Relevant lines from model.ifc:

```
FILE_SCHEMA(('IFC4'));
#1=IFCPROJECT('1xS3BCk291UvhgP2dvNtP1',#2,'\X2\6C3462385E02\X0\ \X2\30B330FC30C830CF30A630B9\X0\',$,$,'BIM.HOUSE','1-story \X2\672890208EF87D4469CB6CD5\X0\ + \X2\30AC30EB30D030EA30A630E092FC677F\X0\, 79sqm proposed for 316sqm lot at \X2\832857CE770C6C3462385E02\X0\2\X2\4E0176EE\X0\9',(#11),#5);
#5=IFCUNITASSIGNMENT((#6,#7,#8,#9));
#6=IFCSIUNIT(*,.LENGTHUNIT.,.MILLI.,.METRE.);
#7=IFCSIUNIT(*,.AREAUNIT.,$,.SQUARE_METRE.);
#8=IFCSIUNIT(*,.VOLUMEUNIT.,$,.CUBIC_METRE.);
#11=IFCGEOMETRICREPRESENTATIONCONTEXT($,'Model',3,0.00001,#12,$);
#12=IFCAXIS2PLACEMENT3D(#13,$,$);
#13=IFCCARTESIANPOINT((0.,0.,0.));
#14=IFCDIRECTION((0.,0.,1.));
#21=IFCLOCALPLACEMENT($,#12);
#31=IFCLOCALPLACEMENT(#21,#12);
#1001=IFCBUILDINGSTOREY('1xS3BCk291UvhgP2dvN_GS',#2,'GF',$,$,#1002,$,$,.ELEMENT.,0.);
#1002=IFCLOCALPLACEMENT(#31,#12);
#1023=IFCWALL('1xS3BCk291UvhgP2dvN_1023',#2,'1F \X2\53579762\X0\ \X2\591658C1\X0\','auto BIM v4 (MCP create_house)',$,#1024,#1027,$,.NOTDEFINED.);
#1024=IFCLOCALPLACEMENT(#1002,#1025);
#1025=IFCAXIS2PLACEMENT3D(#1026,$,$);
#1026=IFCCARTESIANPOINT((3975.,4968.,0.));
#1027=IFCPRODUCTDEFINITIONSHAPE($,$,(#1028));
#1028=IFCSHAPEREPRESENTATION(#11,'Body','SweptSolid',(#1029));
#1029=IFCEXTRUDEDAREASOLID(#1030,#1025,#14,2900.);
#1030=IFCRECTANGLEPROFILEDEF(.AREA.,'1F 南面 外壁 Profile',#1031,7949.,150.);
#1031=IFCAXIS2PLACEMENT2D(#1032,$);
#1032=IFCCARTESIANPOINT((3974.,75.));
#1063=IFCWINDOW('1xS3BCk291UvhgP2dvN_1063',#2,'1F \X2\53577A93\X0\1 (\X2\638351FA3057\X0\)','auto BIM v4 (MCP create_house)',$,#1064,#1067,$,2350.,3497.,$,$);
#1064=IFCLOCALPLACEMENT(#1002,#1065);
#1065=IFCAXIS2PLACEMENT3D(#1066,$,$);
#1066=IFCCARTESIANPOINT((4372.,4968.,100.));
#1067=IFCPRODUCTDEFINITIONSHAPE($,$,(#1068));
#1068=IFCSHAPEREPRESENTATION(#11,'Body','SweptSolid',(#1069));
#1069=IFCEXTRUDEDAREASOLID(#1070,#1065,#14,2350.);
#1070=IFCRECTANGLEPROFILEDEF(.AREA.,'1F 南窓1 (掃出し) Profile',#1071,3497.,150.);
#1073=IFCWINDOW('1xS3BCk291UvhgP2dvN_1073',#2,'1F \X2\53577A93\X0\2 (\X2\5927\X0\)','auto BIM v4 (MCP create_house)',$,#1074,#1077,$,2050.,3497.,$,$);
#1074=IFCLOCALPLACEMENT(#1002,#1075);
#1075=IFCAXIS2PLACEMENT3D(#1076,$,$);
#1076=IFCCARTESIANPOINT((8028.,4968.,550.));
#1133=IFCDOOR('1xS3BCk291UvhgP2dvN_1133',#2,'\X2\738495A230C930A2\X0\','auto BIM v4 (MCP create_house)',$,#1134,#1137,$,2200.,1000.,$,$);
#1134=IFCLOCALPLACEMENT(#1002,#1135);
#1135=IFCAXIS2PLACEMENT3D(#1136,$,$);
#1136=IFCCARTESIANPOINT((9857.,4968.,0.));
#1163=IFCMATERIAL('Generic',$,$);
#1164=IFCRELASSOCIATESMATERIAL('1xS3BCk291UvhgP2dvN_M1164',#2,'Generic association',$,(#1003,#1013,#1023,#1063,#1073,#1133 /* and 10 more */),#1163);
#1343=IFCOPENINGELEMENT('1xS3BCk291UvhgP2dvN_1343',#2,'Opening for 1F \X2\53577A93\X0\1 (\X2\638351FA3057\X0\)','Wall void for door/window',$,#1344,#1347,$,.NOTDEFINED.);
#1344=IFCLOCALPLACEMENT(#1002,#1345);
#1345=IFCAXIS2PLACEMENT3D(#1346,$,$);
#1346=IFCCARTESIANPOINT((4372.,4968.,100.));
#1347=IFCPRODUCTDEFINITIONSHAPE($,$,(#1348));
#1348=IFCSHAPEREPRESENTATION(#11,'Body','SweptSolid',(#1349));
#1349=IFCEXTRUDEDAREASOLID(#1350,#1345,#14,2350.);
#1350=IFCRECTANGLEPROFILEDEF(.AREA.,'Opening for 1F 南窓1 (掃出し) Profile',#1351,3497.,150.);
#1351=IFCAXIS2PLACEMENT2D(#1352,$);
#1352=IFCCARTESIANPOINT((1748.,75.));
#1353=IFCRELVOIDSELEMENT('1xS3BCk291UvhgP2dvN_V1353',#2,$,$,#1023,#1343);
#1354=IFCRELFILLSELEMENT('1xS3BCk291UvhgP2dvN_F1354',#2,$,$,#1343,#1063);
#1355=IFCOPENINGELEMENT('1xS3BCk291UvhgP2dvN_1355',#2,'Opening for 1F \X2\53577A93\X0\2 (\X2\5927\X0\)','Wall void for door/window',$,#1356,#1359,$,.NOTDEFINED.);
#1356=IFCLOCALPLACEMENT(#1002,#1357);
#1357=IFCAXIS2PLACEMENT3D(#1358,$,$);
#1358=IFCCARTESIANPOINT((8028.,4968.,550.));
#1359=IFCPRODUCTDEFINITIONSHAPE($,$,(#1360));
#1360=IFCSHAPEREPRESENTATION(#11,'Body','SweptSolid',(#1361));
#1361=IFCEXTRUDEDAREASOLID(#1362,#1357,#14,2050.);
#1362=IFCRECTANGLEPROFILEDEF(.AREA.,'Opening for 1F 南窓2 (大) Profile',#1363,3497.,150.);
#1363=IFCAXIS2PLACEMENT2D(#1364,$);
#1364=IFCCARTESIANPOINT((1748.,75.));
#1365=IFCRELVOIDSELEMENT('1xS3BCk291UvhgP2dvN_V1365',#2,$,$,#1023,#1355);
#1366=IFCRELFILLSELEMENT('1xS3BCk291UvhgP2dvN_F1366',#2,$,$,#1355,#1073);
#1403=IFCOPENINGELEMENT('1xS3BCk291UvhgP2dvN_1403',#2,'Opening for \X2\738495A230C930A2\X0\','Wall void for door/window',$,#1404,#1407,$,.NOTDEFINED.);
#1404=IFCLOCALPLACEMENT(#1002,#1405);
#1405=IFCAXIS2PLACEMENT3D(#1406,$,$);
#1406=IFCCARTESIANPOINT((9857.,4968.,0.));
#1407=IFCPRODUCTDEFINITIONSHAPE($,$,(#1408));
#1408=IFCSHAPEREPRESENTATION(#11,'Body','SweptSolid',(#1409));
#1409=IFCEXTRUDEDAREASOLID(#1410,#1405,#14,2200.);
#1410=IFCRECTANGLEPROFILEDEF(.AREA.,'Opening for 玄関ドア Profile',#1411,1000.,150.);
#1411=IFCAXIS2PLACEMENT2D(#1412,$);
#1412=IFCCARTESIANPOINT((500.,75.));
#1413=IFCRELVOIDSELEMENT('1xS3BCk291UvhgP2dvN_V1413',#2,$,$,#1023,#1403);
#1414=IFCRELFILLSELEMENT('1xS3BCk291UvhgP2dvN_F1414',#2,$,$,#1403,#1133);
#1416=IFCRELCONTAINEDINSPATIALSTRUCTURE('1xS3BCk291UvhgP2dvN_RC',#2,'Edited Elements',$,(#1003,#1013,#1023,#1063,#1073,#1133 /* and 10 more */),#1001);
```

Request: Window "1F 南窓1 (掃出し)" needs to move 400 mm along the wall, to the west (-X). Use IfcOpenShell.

```python
import ifcopenshell
import ifcopenshell.api.geometry
import ifcopenshell.util.placement
import ifcopenshell.util.unit

model = ifcopenshell.open("model.ifc")
unit_scale = ifcopenshell.util.unit.calculate_unit_scale(model)

window = model.by_id(1063)
opening = window.FillsVoids[0].RelatingOpeningElement
wall = opening.VoidsElements[0].RelatingBuildingElement

wall_matrix = ifcopenshell.util.placement.get_local_placement(wall.ObjectPlacement)
shift = wall_matrix[:3, 0] * -0.4 / unit_scale
before = ifcopenshell.util.placement.get_local_placement(window.ObjectPlacement)[:3, 3].copy()

# The window is not placed relative to its opening, so move both.
for product in (opening, window):
    matrix = ifcopenshell.util.placement.get_local_placement(product.ObjectPlacement)
    matrix[:3, 3] += shift
    ifcopenshell.api.geometry.edit_object_placement(model, product=product, matrix=matrix, is_si=False)

after = ifcopenshell.util.placement.get_local_placement(window.ObjectPlacement)[:3, 3]
print("window moved by", (after - before).round(3) + 0.0)

model.write("model_rev.ifc")
```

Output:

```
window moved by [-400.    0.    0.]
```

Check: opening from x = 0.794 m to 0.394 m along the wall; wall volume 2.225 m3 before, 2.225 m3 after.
